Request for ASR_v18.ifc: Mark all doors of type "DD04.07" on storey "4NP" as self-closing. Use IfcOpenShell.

First a look at what the model holds.

```python
import ifcopenshell
import ifcopenshell.util.element

model = ifcopenshell.open("ASR_v18.ifc")
print(model.schema)
storey = next(s for s in model.by_type("IfcBuildingStorey") if s.Name == "4NP")
doors = [e for e in ifcopenshell.util.element.get_decomposition(storey) if e.is_a("IfcDoor")]
seen = {}
for e in doors:
    element_type = ifcopenshell.util.element.get_type(e)
    key = (element_type.Name if element_type != e and element_type else None, ifcopenshell.util.element.get_pset(e, "Pset_DoorCommon", "SelfClosing"))
    seen[key] = seen.get(key, 0) + 1
for (name, value), count in sorted(seen.items(), key=str):
    print(count, "x", name, "|", value)
```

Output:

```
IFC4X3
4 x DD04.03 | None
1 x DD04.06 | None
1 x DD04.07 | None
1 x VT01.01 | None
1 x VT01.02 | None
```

```python
import ifcopenshell
import ifcopenshell.api.pset
import ifcopenshell.util.element

model = ifcopenshell.open("ASR_v18.ifc")

storey = next(s for s in model.by_type("IfcBuildingStorey") if s.Name == "4NP")
doors = [e for e in ifcopenshell.util.element.get_decomposition(storey) if e.is_a("IfcDoor")]

count = 0
for e in doors:
    element_type = ifcopenshell.util.element.get_type(e)
    if element_type in (None, e) or element_type.Name != "DD04.07":
        continue
    # add_pset returns the element's existing set when there is one.
    pset = ifcopenshell.api.pset.add_pset(model, product=e, name="Pset_DoorCommon")
    ifcopenshell.api.pset.edit_pset(model, pset=pset, properties={"SelfClosing": True})
    count += 1

print(count, "doors updated")

model.write("ASR_v18_v2.ifc")
```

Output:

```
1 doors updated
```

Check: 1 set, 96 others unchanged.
